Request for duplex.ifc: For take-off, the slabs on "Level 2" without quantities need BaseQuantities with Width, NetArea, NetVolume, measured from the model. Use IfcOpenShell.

First a look at what the model holds.

```python
import ifcopenshell
import ifcopenshell.util.element
import ifcopenshell.util.unit

model = ifcopenshell.open("duplex.ifc")
print(model.schema)
for unit_type in ("LENGTHUNIT", "AREAUNIT", "VOLUMEUNIT"):
    print(unit_type, ifcopenshell.util.unit.calculate_unit_scale(model, unit_type))
storey = next(s for s in model.by_type("IfcBuildingStorey") if s.Name == "Level 2")
slabs = [e for e in ifcopenshell.util.element.get_decomposition(storey) if e.is_a("IfcSlab")]
for e in sorted(slabs, key=lambda e: e.id()):
    print(e.id(), e.is_a(), e.Name, list(ifcopenshell.util.element.get_psets(e, qtos_only=True)), sep=" | ")
```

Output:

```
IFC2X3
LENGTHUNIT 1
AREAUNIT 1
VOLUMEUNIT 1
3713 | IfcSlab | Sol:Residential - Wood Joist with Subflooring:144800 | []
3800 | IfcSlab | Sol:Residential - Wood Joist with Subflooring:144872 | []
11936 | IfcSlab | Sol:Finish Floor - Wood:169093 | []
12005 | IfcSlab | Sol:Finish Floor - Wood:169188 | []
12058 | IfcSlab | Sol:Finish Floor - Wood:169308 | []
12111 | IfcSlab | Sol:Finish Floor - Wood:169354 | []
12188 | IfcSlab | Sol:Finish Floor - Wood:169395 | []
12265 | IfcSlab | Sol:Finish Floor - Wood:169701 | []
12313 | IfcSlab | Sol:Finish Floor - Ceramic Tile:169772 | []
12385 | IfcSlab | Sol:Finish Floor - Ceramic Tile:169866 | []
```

```python
import ifcopenshell
import ifcopenshell.api.pset
import ifcopenshell.geom
import ifcopenshell.util.element
import ifcopenshell.util.shape
import ifcopenshell.util.unit

model = ifcopenshell.open("duplex.ifc")
unit_scale = ifcopenshell.util.unit.calculate_unit_scale(model)
area_scale = ifcopenshell.util.unit.calculate_unit_scale(model, "AREAUNIT")
volume_scale = ifcopenshell.util.unit.calculate_unit_scale(model, "VOLUMEUNIT")
settings = ifcopenshell.geom.settings()

storey = next(s for s in model.by_type("IfcBuildingStorey") if s.Name == "Level 2")
slabs = [e for e in ifcopenshell.util.element.get_decomposition(storey) if e.is_a("IfcSlab")]

for e in sorted(slabs, key=lambda e: e.id()):
    if ifcopenshell.util.element.get_psets(e, qtos_only=True, should_inherit=False):
        continue
    # Geometry comes back in metres, in the element's own axes.
    shape = ifcopenshell.geom.create_shape(settings, e)
    values = {
        "Width": ifcopenshell.util.shape.get_z(shape.geometry) / unit_scale,
        "NetArea": ifcopenshell.util.shape.get_footprint_area(shape.geometry) / area_scale,
        "NetVolume": ifcopenshell.util.shape.get_volume(shape.geometry) / volume_scale,
    }
    qto = ifcopenshell.api.pset.add_qto(model, product=e, name="BaseQuantities")
    ifcopenshell.api.pset.edit_qto(model, qto=qto, properties=values)
    print(e.id(), {k: round(v, 3) for k, v in values.items()})

model.write("duplex-out.ifc")
```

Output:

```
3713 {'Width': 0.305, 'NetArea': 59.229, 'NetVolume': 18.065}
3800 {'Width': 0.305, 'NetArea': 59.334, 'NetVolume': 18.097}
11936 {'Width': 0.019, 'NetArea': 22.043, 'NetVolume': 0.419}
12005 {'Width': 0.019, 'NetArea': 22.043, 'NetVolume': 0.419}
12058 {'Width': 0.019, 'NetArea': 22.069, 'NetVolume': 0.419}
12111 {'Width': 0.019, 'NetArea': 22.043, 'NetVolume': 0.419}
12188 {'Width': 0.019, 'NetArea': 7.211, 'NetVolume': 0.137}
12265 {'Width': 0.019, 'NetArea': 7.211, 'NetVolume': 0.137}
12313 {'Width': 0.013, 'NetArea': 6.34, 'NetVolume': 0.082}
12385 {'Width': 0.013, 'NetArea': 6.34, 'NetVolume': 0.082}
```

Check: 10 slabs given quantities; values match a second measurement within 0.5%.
